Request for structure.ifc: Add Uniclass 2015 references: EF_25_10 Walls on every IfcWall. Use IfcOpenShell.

First a look at what the model holds.

```python
import ifcopenshell

model = ifcopenshell.open("structure.ifc")
print(model.schema)
print("classifications:", [c.Name for c in model.by_type("IfcClassification")])
for ifc_class in ("IfcDoor", "IfcRoof", "IfcStair", "IfcWall", "IfcWindow"):
    print(ifc_class, len(model.by_type(ifc_class)))
```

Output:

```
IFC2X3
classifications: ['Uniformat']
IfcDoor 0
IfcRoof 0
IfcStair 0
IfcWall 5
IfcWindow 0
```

```python
import ifcopenshell
import ifcopenshell.api.classification

model = ifcopenshell.open("structure.ifc")

# IFC2X3 requires Source and Edition and has no link from the project to the system.
system = model.create_entity("IfcClassification", Source="NBS", Edition="2015", Name="Uniclass 2015")

codes = {
    "IfcWall": ("EF_25_10", "Walls"),
}
for ifc_class, (code, name) in codes.items():
    products = model.by_type(ifc_class)
    ifcopenshell.api.classification.add_reference(
        model, products=products, classification=system, identification=code, name=name
    )
    print(code, len(products))

model.write("structure_updated.ifc")
```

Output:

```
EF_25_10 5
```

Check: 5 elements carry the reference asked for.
